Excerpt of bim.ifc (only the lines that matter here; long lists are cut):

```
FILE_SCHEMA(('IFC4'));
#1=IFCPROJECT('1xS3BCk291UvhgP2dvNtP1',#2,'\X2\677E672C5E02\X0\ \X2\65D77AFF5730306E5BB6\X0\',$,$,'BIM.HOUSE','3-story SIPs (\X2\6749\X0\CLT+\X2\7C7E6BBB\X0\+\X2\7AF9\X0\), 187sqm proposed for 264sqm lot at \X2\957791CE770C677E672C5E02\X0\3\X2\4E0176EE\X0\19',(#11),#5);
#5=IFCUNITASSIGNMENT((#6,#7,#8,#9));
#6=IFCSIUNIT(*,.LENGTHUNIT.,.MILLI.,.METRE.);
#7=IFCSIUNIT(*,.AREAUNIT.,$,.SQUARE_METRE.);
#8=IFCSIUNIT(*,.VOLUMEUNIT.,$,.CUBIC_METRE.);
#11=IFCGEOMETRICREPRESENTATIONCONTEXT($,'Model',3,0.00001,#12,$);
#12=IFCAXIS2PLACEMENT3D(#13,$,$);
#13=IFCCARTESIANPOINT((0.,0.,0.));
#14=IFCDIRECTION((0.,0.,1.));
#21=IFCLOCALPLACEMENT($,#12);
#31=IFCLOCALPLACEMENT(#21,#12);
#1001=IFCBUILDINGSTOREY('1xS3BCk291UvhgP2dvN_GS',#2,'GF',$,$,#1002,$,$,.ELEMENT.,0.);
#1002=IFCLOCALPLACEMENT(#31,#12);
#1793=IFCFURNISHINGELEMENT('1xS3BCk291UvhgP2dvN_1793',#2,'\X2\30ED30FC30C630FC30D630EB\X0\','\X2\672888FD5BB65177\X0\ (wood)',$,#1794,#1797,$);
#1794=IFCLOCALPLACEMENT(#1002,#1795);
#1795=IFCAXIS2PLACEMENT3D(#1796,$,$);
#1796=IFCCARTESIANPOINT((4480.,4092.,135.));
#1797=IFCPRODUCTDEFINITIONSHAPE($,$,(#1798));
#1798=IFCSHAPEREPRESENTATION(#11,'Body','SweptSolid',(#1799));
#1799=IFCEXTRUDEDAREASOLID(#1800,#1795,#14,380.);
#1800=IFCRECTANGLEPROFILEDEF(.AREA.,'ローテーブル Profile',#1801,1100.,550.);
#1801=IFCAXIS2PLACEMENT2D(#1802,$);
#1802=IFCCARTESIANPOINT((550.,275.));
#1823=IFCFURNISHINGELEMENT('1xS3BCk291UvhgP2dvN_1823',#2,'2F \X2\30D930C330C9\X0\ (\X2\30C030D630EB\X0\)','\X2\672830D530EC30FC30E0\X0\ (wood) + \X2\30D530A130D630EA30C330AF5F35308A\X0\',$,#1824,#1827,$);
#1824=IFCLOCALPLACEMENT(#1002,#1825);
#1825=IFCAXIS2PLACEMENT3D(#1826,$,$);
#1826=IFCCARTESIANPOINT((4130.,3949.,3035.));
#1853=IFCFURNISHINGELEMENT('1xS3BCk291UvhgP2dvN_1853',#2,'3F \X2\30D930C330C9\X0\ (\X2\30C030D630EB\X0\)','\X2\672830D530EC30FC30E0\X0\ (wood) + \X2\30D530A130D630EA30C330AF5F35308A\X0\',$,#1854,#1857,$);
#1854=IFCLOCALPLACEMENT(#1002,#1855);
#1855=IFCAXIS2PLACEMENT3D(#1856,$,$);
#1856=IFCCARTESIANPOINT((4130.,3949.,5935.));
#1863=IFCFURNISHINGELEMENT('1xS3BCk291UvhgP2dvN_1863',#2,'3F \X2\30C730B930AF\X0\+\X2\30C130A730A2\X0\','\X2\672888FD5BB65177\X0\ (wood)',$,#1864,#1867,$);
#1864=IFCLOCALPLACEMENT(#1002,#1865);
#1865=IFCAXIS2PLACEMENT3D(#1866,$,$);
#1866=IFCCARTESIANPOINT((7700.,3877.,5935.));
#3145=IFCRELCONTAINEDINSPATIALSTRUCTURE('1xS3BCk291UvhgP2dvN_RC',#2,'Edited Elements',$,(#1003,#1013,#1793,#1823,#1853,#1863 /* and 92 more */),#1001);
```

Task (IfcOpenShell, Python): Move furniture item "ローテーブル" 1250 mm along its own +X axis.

```python
import ifcopenshell
import ifcopenshell.api.geometry
import ifcopenshell.util.placement
import ifcopenshell.util.unit

model = ifcopenshell.open("bim.ifc")
unit_scale = ifcopenshell.util.unit.calculate_unit_scale(model)

item = model.by_guid("1xS3BCk291UvhgP2dvN_1793")
matrix = ifcopenshell.util.placement.get_local_placement(item.ObjectPlacement)
matrix[:3, 3] += matrix[:3, 0] * 1.25 / unit_scale
ifcopenshell.api.geometry.edit_object_placement(model, product=item, matrix=matrix, is_si=False)

print(ifcopenshell.util.placement.get_local_placement(item.ObjectPlacement).round(3) + 0.0)

model.write("bim-out.ifc")
```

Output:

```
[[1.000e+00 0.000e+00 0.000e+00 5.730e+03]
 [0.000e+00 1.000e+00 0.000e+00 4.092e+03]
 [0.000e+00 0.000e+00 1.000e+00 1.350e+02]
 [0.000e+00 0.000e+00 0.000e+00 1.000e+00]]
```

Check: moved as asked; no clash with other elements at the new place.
